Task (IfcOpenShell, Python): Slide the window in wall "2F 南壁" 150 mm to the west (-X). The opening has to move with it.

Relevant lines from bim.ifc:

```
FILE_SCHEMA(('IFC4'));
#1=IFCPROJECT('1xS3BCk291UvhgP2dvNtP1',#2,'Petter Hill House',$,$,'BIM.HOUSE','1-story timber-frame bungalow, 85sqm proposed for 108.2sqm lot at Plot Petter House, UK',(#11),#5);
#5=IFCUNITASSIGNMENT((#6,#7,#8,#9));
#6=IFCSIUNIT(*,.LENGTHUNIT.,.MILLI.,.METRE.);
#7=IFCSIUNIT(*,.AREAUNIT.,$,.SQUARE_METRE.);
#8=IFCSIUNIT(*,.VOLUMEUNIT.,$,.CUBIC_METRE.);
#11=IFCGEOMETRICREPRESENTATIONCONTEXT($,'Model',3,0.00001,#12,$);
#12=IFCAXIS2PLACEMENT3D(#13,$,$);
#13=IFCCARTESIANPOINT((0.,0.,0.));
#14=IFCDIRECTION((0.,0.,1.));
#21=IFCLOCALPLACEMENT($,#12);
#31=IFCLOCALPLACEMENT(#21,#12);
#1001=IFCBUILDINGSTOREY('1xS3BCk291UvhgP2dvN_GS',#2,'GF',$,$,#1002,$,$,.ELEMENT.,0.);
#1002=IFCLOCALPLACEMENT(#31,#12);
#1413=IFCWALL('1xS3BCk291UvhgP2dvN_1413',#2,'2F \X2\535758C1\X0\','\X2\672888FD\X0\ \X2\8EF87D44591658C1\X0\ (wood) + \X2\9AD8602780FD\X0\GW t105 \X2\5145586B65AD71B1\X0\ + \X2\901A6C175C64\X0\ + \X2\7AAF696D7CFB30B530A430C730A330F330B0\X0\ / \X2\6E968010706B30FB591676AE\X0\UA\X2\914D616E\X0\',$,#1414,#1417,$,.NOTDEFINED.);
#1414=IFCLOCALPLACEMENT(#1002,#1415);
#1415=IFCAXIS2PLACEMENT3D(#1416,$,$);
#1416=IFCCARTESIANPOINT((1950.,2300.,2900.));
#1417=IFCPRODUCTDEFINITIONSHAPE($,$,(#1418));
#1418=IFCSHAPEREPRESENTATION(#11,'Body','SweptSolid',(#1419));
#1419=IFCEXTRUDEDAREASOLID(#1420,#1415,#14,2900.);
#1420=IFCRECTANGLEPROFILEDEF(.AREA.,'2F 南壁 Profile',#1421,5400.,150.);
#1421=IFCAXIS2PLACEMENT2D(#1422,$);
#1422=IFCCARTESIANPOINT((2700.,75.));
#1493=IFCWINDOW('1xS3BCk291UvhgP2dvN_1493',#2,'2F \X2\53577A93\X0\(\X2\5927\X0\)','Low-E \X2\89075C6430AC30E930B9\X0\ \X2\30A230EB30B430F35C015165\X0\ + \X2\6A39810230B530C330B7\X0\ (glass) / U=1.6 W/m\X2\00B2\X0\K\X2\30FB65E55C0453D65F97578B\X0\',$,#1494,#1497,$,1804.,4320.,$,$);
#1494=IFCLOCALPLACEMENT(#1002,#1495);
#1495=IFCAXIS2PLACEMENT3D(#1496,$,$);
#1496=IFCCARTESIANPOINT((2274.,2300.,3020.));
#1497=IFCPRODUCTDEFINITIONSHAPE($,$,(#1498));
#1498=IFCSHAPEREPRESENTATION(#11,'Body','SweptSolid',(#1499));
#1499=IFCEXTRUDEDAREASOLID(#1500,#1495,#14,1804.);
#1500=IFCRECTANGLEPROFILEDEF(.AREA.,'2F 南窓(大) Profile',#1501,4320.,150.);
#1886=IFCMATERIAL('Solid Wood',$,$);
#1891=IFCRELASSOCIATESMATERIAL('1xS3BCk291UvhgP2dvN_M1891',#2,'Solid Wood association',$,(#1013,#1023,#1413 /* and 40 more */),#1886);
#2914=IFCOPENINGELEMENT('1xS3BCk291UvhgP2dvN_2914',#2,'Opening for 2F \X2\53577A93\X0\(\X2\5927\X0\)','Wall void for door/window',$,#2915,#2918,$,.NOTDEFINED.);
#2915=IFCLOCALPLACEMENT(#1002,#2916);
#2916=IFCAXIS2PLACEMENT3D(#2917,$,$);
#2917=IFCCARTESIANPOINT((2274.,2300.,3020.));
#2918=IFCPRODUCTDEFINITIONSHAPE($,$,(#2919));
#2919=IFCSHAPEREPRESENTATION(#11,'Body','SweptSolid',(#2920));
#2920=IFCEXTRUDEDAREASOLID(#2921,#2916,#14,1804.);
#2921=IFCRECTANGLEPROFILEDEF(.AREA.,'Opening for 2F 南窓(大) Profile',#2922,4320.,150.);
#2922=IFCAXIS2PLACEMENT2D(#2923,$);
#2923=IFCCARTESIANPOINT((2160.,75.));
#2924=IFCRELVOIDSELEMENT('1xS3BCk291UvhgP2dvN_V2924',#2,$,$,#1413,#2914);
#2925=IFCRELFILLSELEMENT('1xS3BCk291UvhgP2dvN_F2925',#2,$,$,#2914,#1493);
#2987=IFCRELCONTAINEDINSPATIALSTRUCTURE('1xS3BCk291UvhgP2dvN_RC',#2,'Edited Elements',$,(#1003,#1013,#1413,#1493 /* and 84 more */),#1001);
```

```python
import ifcopenshell
import ifcopenshell.api.geometry
import ifcopenshell.util.placement

model = ifcopenshell.open("bim.ifc")

window = model.by_guid("1xS3BCk291UvhgP2dvN_1493")
opening = window.FillsVoids[0].RelatingOpeningElement
wall = opening.VoidsElements[0].RelatingBuildingElement

wall_matrix = ifcopenshell.util.placement.get_local_placement(wall.ObjectPlacement)
shift = wall_matrix[:3, 0] * -150.0
before = ifcopenshell.util.placement.get_local_placement(window.ObjectPlacement)[:3, 3].copy()

# The window is not placed relative to its opening, so move both.
for product in (opening, window):
    matrix = ifcopenshell.util.placement.get_local_placement(product.ObjectPlacement)
    matrix[:3, 3] += shift
    ifcopenshell.api.geometry.edit_object_placement(model, product=product, matrix=matrix, is_si=False)

after = ifcopenshell.util.placement.get_local_placement(window.ObjectPlacement)[:3, 3]
print("window moved by", (after - before).round(3) + 0.0)

model.write("bim-out.ifc")
```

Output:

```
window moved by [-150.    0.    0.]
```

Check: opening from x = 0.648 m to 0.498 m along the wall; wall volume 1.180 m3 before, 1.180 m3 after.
